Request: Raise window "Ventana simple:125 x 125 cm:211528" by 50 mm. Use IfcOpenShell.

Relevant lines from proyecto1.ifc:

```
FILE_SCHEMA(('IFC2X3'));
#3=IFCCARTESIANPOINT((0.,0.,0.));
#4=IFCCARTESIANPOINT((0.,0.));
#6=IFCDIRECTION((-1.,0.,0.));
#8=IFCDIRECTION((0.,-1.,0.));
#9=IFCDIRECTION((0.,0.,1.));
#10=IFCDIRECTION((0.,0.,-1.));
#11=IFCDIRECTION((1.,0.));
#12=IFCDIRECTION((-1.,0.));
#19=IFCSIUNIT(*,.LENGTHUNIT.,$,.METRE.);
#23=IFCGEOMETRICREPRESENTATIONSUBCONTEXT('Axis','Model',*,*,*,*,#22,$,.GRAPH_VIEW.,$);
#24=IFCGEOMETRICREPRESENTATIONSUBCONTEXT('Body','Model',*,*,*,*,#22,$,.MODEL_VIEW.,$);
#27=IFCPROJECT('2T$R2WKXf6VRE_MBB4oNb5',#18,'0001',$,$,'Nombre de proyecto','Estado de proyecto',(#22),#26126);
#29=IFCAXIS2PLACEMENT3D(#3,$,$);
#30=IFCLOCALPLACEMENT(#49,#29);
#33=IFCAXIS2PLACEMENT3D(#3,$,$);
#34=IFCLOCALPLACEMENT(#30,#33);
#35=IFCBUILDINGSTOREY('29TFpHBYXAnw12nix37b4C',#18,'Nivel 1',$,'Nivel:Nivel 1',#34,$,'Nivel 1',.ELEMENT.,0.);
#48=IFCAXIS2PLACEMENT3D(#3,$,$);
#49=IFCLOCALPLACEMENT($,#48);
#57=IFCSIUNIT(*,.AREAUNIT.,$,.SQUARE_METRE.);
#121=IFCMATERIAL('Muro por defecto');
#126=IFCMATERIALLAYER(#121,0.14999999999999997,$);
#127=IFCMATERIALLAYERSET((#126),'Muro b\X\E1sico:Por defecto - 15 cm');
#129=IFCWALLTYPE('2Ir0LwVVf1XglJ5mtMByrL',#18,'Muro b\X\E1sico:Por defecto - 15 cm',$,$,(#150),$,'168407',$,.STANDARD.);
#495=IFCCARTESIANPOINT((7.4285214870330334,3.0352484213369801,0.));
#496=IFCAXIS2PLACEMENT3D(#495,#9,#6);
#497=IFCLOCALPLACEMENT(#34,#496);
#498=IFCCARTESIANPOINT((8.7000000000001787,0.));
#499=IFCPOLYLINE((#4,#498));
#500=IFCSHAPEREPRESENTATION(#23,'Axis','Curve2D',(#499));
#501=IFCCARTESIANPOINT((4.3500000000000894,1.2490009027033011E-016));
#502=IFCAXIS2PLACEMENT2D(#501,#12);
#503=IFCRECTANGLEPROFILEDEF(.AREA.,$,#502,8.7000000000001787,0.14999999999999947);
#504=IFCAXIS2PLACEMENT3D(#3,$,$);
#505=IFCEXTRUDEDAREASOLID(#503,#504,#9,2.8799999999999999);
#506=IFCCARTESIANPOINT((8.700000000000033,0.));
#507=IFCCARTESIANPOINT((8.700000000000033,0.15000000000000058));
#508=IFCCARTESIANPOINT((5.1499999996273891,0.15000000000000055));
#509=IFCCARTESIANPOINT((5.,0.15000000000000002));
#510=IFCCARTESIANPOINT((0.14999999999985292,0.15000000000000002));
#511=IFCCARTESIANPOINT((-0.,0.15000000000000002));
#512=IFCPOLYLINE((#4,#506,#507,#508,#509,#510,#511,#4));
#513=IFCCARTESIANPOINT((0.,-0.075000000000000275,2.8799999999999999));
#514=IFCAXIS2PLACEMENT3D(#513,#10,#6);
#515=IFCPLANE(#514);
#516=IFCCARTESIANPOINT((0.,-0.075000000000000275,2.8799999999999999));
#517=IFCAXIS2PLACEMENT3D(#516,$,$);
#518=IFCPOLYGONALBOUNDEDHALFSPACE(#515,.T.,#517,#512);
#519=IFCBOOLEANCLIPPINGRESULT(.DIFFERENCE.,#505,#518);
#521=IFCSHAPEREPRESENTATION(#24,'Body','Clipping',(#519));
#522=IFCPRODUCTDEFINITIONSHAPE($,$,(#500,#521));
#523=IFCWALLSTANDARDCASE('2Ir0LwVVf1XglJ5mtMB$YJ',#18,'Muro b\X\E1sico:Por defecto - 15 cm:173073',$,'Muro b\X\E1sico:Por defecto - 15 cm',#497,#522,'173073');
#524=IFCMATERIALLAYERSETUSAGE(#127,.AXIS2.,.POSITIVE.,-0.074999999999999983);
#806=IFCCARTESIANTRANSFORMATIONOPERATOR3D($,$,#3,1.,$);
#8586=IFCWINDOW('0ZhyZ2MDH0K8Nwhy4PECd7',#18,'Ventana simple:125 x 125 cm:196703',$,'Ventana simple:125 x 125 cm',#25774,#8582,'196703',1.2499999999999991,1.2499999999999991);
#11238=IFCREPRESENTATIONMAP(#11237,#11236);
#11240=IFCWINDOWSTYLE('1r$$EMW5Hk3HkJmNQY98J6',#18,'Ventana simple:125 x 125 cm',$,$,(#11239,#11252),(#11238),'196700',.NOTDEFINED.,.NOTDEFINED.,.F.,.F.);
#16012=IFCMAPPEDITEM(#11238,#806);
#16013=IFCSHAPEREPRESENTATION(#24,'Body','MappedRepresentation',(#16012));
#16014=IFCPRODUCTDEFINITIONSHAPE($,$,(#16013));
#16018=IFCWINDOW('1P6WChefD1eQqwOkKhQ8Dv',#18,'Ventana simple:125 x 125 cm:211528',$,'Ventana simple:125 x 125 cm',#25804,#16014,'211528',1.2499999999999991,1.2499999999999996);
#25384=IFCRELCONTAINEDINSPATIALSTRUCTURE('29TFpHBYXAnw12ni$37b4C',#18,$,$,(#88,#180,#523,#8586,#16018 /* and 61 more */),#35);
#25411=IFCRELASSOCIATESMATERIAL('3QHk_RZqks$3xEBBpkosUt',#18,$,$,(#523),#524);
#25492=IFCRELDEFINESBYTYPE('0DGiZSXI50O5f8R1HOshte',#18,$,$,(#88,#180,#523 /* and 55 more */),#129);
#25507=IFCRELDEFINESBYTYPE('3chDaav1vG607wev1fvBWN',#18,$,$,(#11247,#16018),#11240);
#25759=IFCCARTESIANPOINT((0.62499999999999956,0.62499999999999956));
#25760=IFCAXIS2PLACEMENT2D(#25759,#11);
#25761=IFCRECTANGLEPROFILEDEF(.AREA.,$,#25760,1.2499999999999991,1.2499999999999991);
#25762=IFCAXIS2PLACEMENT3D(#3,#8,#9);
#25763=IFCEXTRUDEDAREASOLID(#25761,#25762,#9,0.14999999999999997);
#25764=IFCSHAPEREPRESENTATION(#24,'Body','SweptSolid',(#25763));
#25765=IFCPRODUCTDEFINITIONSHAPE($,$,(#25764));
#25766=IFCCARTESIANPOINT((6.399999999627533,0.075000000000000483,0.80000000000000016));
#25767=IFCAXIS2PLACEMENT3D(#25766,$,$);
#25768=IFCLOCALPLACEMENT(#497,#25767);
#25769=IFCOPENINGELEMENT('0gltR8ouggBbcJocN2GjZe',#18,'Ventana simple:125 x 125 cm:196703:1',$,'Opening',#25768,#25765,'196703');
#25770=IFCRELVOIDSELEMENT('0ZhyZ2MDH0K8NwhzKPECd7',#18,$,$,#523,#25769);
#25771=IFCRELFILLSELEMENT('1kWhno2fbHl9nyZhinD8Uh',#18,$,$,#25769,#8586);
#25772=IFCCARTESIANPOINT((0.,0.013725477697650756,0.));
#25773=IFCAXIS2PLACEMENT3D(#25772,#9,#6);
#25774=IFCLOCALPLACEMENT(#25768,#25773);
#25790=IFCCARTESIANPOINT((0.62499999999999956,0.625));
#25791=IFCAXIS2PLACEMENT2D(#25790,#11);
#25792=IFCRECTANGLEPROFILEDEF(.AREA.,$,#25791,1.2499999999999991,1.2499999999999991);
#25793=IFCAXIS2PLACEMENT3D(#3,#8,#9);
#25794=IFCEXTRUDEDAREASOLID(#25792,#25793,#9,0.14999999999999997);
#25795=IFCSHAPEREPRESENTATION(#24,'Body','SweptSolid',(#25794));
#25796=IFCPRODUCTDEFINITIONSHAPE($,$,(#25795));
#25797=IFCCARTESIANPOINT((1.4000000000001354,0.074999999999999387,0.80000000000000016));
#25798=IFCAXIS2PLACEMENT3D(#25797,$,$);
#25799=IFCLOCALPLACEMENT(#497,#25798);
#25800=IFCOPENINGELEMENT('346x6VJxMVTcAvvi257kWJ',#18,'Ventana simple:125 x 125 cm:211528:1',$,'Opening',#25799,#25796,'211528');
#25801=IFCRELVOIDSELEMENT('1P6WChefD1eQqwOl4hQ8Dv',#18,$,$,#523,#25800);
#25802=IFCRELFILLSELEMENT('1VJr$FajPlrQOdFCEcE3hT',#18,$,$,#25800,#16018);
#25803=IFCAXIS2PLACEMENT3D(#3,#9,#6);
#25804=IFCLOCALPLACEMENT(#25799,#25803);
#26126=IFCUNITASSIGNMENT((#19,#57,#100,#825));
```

```python
import numpy as np
import ifcopenshell
import ifcopenshell.api.geometry
import ifcopenshell.util.placement
import ifcopenshell.util.unit

model = ifcopenshell.open("proyecto1.ifc")
unit_scale = ifcopenshell.util.unit.calculate_unit_scale(model)

window = model.by_guid("1P6WChefD1eQqwOkKhQ8Dv")
opening = window.FillsVoids[0].RelatingOpeningElement
dz = 0.05 / unit_scale

shift = np.array([0.0, 0.0, dz])
# The window is placed relative to its opening, so it follows when the opening moves.
matrix = ifcopenshell.util.placement.get_local_placement(opening.ObjectPlacement)
matrix[:3, 3] += shift
ifcopenshell.api.geometry.edit_object_placement(
    model, product=opening, matrix=matrix, is_si=False, should_transform_children=True
)

print(f"moved by {dz * unit_scale:+.3f} m")

model.write("proyecto1_v2.ifc")
```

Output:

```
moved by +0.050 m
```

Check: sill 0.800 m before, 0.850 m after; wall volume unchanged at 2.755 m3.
